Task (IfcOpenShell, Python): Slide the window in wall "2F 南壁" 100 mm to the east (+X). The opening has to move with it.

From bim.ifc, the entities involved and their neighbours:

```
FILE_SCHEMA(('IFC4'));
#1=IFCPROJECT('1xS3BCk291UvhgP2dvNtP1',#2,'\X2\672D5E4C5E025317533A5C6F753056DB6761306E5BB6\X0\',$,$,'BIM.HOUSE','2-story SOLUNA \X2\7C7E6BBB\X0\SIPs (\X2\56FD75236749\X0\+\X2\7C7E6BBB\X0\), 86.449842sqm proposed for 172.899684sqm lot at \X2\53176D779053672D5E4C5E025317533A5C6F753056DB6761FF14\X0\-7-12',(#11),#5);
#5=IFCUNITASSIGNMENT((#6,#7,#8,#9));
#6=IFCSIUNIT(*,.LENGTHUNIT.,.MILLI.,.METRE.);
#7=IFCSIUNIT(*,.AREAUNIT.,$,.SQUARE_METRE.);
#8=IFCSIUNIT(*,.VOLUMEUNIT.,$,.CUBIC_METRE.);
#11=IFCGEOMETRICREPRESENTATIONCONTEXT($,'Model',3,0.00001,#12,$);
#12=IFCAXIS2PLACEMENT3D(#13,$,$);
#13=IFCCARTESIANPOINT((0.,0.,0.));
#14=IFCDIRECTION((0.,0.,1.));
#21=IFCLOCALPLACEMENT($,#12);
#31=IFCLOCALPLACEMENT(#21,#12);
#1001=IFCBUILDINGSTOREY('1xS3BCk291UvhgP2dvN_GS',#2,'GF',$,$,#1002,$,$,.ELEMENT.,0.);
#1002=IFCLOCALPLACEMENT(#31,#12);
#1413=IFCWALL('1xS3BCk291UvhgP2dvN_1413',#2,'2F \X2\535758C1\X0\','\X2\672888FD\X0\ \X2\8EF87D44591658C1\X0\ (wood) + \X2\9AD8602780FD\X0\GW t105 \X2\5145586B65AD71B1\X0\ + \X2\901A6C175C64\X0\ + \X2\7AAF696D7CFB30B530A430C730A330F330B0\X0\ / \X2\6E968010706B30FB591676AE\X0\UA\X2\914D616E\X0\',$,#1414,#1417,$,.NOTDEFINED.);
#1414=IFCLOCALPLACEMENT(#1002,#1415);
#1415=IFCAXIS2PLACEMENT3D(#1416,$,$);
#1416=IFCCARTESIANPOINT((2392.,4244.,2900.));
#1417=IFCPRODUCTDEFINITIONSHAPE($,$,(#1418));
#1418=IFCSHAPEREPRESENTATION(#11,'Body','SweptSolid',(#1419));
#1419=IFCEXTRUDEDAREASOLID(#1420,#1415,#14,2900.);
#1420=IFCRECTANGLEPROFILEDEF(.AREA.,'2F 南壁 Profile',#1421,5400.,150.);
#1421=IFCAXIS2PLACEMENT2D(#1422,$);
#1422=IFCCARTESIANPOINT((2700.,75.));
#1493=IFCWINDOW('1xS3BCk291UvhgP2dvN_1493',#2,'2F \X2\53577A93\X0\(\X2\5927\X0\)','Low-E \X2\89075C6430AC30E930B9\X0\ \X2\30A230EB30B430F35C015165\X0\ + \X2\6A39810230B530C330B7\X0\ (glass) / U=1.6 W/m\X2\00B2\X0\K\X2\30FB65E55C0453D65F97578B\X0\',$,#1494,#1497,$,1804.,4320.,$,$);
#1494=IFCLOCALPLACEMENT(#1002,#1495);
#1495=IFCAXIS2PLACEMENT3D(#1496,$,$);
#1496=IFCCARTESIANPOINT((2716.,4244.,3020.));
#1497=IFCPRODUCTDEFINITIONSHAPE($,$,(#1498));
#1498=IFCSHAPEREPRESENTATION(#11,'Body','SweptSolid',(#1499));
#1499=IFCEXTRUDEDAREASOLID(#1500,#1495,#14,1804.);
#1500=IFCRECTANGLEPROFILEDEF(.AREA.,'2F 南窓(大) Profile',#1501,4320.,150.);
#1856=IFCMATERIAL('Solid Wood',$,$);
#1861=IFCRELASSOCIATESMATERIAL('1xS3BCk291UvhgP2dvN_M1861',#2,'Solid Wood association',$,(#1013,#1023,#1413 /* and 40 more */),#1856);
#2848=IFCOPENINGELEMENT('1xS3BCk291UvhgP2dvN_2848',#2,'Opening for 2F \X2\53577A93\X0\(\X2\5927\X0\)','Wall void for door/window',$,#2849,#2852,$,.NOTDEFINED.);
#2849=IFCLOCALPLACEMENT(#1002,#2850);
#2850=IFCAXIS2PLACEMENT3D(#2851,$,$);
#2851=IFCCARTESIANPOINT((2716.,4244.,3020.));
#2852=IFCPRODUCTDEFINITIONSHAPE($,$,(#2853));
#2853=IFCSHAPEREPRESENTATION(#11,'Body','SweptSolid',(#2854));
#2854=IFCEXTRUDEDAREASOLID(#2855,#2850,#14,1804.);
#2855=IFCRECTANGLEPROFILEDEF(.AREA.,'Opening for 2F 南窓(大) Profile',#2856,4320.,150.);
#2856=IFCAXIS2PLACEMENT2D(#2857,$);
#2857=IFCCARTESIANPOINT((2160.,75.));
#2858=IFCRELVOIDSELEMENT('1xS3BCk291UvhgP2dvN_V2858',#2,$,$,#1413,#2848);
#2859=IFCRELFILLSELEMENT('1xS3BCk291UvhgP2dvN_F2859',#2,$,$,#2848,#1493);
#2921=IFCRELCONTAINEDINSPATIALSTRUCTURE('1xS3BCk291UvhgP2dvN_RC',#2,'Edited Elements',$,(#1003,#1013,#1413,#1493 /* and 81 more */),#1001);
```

```python
import ifcopenshell
import ifcopenshell.api.geometry
import ifcopenshell.util.placement
import ifcopenshell.util.unit

model = ifcopenshell.open("bim.ifc")
unit_scale = ifcopenshell.util.unit.calculate_unit_scale(model)

window = model.by_id(1493)
opening = window.FillsVoids[0].RelatingOpeningElement
wall = opening.VoidsElements[0].RelatingBuildingElement

wall_matrix = ifcopenshell.util.placement.get_local_placement(wall.ObjectPlacement)
shift = wall_matrix[:3, 0] * 0.1 / unit_scale
before = ifcopenshell.util.placement.get_local_placement(window.ObjectPlacement)[:3, 3].copy()

# The window is not placed relative to its opening, so move both.
for product in (opening, window):
    matrix = ifcopenshell.util.placement.get_local_placement(product.ObjectPlacement)
    matrix[:3, 3] += shift
    ifcopenshell.api.geometry.edit_object_placement(model, product=product, matrix=matrix, is_si=False)

after = ifcopenshell.util.placement.get_local_placement(window.ObjectPlacement)[:3, 3]
print("window moved by", (after - before).round(3) + 0.0)

model.write("bim-out.ifc")
```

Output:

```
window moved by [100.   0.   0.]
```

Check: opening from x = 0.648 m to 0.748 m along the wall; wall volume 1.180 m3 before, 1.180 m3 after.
